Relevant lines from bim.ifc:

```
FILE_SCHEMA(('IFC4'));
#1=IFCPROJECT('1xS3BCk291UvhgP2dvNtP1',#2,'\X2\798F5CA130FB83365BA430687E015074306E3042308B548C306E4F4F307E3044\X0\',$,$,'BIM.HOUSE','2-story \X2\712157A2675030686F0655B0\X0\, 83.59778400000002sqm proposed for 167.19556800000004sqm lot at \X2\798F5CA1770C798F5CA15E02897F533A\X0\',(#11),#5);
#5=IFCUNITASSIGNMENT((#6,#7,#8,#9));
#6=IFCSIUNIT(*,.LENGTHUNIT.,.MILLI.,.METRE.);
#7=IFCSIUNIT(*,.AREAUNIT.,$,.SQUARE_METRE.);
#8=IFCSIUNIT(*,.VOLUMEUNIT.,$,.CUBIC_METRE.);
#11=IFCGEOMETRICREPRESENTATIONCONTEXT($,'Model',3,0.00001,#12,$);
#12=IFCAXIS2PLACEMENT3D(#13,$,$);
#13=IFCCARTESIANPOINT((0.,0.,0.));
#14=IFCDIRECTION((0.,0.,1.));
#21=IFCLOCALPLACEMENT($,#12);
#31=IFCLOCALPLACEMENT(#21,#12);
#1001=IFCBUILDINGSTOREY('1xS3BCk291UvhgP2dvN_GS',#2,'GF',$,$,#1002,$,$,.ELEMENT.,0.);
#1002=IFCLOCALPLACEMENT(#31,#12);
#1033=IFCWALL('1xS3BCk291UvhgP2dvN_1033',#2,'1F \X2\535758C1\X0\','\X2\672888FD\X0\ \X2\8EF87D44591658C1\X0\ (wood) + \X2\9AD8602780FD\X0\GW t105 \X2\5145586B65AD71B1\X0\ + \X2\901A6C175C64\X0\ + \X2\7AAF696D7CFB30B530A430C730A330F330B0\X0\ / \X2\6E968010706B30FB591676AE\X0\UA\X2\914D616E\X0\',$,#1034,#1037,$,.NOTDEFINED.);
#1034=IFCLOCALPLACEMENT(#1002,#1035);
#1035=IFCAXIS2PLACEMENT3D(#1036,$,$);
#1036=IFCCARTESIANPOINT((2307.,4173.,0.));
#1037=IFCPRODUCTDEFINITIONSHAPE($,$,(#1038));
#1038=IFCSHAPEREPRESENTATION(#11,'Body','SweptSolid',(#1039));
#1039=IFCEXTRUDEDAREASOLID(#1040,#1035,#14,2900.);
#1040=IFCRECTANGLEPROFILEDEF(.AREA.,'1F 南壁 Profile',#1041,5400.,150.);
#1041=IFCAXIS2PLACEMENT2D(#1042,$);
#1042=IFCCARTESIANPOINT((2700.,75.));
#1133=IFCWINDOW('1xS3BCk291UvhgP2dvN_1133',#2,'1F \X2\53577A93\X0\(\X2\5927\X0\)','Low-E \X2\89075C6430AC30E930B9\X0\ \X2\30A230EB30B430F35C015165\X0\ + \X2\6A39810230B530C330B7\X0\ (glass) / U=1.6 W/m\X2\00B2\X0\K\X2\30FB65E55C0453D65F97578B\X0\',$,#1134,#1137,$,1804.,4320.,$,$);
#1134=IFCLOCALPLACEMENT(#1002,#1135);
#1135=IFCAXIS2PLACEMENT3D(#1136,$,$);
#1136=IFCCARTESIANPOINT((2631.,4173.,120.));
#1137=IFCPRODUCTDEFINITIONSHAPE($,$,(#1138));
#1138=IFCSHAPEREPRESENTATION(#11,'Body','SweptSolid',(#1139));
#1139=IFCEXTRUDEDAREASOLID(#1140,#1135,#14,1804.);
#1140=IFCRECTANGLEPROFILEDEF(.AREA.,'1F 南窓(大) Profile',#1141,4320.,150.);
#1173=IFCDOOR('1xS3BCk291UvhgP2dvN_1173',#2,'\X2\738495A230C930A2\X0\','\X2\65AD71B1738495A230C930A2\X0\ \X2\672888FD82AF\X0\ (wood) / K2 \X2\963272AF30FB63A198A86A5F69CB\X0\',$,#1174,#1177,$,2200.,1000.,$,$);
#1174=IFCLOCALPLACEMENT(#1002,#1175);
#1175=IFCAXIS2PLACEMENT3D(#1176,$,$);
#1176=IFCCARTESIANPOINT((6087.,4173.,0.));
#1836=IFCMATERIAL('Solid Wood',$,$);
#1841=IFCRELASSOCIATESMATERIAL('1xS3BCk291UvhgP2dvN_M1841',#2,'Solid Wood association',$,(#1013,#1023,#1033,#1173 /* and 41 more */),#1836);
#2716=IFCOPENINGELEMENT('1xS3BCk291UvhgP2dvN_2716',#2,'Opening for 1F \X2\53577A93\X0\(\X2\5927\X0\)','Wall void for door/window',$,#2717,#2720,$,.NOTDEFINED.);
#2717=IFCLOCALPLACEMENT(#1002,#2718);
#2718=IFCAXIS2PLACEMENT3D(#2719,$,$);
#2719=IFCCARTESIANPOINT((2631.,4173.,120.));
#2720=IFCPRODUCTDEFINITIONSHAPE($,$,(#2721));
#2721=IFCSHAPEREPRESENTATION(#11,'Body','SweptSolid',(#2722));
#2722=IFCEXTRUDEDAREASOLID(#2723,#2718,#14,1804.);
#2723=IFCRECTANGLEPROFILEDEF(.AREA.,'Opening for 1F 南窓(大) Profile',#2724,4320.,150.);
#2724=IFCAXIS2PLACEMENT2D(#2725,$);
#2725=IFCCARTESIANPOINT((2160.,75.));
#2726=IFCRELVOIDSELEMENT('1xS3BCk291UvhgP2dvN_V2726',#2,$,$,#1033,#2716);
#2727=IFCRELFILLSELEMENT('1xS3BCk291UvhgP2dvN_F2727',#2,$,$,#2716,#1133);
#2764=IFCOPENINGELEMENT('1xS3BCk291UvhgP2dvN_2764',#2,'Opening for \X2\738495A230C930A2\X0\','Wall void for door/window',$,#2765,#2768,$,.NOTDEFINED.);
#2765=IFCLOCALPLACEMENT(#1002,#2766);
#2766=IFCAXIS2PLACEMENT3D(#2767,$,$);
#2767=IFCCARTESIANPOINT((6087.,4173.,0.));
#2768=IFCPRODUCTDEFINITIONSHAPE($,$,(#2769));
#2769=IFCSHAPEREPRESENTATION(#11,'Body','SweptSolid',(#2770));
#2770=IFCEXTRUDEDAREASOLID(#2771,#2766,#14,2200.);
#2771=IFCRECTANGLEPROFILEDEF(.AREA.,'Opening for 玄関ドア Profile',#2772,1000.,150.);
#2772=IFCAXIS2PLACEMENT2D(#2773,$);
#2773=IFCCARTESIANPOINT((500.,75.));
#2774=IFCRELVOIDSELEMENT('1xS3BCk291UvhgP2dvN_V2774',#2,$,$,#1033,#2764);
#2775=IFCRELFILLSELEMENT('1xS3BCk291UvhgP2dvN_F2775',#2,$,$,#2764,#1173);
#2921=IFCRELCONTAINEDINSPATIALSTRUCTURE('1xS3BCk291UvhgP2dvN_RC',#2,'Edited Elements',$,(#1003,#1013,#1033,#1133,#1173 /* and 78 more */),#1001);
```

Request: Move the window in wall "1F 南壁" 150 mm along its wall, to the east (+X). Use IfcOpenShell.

```python
import ifcopenshell
import ifcopenshell.api.geometry
import ifcopenshell.util.placement

model = ifcopenshell.open("bim.ifc")

window = model.by_guid("1xS3BCk291UvhgP2dvN_1133")
opening = window.FillsVoids[0].RelatingOpeningElement
wall = opening.VoidsElements[0].RelatingBuildingElement

wall_matrix = ifcopenshell.util.placement.get_local_placement(wall.ObjectPlacement)
shift = wall_matrix[:3, 0] * 150.0
before = ifcopenshell.util.placement.get_local_placement(window.ObjectPlacement)[:3, 3].copy()

# The window is not placed relative to its opening, so move both.
for product in (opening, window):
    matrix = ifcopenshell.util.placement.get_local_placement(product.ObjectPlacement)
    matrix[:3, 3] += shift
    ifcopenshell.api.geometry.edit_object_placement(model, product=product, matrix=matrix, is_si=False)

after = ifcopenshell.util.placement.get_local_placement(window.ObjectPlacement)[:3, 3]
print("window moved by", (after - before).round(3) + 0.0)

model.write("bim_updated.ifc")
```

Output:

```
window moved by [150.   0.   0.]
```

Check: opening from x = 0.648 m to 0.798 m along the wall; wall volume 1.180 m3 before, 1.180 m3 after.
